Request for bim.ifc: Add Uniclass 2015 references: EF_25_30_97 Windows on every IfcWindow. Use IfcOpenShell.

First a look at what the model holds.

```python
import ifcopenshell

model = ifcopenshell.open("bim.ifc")
print(model.schema)
print("classifications:", [c.Name for c in model.by_type("IfcClassification")])
for ifc_class in ("IfcDoor", "IfcRoof", "IfcStair", "IfcWall", "IfcWindow"):
    print(ifc_class, len(model.by_type(ifc_class)))
```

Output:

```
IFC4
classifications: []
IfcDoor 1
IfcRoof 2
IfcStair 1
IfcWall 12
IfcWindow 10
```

```python
import ifcopenshell
import ifcopenshell.api.classification

model = ifcopenshell.open("bim.ifc")

system = ifcopenshell.api.classification.add_classification(model, classification="Uniclass 2015")

codes = {
    "IfcWindow": ("EF_25_30_97", "Windows"),
}
for ifc_class, (code, name) in codes.items():
    products = model.by_type(ifc_class)
    ifcopenshell.api.classification.add_reference(
        model, products=products, classification=system, identification=code, name=name
    )
    print(code, len(products))

model.write("bim_edited.ifc")
```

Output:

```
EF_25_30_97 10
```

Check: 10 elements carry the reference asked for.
